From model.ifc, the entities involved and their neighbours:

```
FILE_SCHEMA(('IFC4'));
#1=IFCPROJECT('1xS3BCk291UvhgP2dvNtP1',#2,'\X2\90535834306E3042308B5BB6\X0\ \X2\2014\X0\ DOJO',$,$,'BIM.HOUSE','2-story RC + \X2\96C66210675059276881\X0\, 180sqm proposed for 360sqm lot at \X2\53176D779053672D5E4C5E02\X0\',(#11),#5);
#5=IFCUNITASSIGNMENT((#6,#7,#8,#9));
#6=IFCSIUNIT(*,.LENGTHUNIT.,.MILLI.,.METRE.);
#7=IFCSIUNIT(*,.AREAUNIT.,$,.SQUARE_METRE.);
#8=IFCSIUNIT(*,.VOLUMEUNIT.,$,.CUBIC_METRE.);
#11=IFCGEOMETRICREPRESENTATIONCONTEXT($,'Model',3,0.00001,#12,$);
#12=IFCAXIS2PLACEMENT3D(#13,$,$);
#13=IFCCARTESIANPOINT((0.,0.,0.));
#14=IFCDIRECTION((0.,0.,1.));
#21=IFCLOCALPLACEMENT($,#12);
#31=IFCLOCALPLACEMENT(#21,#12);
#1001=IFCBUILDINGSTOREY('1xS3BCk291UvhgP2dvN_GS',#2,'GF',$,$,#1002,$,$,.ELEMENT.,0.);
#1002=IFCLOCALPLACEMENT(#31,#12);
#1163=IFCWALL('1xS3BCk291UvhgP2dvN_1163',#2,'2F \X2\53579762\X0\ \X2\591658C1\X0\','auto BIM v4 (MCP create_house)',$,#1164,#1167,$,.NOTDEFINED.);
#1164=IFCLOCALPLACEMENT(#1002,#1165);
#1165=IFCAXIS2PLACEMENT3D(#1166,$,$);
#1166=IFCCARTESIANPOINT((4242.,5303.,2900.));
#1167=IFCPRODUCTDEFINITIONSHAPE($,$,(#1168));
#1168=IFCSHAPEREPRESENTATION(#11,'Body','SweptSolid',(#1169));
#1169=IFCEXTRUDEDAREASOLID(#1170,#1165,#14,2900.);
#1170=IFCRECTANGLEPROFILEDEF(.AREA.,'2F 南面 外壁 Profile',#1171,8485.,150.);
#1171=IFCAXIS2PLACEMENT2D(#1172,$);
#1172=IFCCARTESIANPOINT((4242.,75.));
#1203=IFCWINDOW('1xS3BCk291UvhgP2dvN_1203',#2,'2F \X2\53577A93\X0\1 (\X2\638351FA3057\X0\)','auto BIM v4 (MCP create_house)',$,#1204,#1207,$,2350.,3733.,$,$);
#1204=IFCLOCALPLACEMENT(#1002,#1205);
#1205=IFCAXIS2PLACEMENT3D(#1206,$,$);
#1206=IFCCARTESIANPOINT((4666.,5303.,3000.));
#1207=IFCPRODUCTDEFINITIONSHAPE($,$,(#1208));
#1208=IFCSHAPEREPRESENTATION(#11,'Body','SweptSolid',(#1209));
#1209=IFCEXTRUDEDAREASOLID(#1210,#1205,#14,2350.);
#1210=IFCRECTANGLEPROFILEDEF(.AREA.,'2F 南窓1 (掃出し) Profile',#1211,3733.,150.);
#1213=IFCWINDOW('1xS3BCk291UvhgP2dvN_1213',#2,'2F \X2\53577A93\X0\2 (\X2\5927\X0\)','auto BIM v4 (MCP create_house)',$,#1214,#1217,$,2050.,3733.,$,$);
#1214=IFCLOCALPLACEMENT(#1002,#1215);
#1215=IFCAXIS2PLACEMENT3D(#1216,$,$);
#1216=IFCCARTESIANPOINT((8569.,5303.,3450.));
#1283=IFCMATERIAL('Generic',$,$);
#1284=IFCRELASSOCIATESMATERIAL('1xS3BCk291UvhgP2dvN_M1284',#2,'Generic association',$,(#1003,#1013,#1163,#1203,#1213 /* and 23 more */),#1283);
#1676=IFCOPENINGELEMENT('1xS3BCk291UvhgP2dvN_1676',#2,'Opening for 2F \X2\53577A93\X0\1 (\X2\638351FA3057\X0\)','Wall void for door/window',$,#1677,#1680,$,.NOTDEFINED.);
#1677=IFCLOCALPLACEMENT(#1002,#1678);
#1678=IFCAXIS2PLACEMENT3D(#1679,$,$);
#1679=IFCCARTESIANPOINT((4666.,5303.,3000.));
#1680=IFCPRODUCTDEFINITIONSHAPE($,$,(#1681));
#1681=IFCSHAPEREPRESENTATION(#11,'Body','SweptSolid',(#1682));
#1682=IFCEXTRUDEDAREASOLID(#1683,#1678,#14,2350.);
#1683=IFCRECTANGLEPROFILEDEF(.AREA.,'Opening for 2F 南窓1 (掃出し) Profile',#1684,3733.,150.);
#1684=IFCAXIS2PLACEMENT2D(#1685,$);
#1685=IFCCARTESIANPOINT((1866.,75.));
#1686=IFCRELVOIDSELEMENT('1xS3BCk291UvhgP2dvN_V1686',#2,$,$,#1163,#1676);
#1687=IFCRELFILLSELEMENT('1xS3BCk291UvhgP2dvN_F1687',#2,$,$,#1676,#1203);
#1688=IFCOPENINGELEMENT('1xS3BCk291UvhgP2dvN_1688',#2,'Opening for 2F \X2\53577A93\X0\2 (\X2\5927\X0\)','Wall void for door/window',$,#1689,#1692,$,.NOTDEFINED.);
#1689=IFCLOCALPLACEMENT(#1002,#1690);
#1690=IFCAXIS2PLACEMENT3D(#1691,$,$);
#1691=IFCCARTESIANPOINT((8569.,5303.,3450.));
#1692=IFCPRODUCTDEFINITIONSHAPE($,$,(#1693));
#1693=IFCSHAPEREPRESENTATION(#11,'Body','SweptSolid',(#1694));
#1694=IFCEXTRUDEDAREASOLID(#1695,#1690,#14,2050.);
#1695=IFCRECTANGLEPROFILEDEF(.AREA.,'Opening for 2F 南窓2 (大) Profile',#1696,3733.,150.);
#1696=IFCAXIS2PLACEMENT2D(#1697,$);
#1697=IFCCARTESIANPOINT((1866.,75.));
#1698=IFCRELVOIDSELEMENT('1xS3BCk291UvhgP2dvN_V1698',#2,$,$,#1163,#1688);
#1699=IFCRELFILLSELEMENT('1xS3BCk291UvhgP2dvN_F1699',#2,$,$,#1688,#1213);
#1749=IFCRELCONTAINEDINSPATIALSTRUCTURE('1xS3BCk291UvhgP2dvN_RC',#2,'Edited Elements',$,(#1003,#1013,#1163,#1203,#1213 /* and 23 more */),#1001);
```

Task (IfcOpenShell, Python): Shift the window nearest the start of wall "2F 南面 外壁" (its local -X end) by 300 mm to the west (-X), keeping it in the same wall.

```python
import ifcopenshell
import ifcopenshell.api.geometry
import ifcopenshell.util.placement
import ifcopenshell.util.unit

model = ifcopenshell.open("model.ifc")
unit_scale = ifcopenshell.util.unit.calculate_unit_scale(model)

window = model.by_id(1203)
opening = window.FillsVoids[0].RelatingOpeningElement
wall = opening.VoidsElements[0].RelatingBuildingElement

wall_matrix = ifcopenshell.util.placement.get_local_placement(wall.ObjectPlacement)
shift = wall_matrix[:3, 0] * -0.3 / unit_scale
before = ifcopenshell.util.placement.get_local_placement(window.ObjectPlacement)[:3, 3].copy()

# The window is not placed relative to its opening, so move both.
for product in (opening, window):
    matrix = ifcopenshell.util.placement.get_local_placement(product.ObjectPlacement)
    matrix[:3, 3] += shift
    ifcopenshell.api.geometry.edit_object_placement(model, product=product, matrix=matrix, is_si=False)

after = ifcopenshell.util.placement.get_local_placement(window.ObjectPlacement)[:3, 3]
print("window moved by", (after - before).round(3) + 0.0)

model.write("model_updated.ifc")
```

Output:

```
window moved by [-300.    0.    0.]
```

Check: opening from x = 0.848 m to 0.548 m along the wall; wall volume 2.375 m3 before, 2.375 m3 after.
